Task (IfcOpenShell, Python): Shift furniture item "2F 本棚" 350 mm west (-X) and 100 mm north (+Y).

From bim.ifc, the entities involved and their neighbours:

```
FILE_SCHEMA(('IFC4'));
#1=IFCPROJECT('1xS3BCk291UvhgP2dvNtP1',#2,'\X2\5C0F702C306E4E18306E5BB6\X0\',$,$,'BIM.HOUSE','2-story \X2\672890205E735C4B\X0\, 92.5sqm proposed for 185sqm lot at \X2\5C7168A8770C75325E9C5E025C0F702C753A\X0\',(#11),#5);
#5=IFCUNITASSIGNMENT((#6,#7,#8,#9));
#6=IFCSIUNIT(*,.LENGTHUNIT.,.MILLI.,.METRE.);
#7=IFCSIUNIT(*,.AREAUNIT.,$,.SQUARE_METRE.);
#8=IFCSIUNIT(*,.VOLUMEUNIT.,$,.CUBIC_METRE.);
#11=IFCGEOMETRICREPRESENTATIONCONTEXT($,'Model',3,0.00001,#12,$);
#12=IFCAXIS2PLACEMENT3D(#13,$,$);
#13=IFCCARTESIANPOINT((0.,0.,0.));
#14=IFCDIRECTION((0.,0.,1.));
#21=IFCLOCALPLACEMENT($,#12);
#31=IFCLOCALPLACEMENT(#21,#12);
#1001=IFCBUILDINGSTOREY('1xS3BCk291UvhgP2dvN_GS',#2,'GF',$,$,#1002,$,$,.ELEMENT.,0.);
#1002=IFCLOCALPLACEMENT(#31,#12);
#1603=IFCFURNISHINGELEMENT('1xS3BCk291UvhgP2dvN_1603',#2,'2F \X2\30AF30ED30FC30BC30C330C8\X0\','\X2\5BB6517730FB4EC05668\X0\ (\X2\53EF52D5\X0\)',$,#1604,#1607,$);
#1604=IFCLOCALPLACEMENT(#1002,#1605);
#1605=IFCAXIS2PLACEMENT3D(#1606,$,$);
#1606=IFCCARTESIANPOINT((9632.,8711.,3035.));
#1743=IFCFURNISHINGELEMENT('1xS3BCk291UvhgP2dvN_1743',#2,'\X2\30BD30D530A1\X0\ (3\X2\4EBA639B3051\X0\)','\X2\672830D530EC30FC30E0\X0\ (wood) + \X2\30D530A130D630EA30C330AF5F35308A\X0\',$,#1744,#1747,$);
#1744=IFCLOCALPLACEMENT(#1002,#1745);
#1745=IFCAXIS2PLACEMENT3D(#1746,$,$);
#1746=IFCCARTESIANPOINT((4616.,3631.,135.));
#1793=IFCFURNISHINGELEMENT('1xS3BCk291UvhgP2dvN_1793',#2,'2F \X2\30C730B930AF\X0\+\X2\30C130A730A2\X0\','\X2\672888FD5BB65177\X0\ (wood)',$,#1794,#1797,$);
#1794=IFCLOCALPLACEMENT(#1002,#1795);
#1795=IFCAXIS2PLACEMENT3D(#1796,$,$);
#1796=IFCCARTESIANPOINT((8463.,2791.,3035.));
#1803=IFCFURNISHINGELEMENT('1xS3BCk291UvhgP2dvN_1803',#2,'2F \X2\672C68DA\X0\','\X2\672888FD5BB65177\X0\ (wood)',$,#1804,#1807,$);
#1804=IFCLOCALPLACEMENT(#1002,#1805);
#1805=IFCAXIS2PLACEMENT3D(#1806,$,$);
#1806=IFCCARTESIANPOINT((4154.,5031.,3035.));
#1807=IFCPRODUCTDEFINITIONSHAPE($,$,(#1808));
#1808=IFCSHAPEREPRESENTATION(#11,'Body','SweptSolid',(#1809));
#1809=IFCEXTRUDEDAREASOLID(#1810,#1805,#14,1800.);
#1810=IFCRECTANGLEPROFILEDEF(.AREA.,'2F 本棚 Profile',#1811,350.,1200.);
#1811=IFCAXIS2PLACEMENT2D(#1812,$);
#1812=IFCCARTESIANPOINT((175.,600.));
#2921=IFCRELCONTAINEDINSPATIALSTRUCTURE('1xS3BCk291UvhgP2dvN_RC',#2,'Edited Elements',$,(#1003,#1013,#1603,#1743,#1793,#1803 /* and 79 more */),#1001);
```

```python
import ifcopenshell
import ifcopenshell.api.geometry
import ifcopenshell.util.placement
import ifcopenshell.util.unit

model = ifcopenshell.open("bim.ifc")
unit_scale = ifcopenshell.util.unit.calculate_unit_scale(model)

item = model.by_id(1803)
matrix = ifcopenshell.util.placement.get_local_placement(item.ObjectPlacement)
matrix[0, 3] -= 0.35 / unit_scale
matrix[1, 3] += 0.1 / unit_scale
ifcopenshell.api.geometry.edit_object_placement(model, product=item, matrix=matrix, is_si=False)

print(ifcopenshell.util.placement.get_local_placement(item.ObjectPlacement).round(3) + 0.0)

model.write("bim_rev.ifc")
```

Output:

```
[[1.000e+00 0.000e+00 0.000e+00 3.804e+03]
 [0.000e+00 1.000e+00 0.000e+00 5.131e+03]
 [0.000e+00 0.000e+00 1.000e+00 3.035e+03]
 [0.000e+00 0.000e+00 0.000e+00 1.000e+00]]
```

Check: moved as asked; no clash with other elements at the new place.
